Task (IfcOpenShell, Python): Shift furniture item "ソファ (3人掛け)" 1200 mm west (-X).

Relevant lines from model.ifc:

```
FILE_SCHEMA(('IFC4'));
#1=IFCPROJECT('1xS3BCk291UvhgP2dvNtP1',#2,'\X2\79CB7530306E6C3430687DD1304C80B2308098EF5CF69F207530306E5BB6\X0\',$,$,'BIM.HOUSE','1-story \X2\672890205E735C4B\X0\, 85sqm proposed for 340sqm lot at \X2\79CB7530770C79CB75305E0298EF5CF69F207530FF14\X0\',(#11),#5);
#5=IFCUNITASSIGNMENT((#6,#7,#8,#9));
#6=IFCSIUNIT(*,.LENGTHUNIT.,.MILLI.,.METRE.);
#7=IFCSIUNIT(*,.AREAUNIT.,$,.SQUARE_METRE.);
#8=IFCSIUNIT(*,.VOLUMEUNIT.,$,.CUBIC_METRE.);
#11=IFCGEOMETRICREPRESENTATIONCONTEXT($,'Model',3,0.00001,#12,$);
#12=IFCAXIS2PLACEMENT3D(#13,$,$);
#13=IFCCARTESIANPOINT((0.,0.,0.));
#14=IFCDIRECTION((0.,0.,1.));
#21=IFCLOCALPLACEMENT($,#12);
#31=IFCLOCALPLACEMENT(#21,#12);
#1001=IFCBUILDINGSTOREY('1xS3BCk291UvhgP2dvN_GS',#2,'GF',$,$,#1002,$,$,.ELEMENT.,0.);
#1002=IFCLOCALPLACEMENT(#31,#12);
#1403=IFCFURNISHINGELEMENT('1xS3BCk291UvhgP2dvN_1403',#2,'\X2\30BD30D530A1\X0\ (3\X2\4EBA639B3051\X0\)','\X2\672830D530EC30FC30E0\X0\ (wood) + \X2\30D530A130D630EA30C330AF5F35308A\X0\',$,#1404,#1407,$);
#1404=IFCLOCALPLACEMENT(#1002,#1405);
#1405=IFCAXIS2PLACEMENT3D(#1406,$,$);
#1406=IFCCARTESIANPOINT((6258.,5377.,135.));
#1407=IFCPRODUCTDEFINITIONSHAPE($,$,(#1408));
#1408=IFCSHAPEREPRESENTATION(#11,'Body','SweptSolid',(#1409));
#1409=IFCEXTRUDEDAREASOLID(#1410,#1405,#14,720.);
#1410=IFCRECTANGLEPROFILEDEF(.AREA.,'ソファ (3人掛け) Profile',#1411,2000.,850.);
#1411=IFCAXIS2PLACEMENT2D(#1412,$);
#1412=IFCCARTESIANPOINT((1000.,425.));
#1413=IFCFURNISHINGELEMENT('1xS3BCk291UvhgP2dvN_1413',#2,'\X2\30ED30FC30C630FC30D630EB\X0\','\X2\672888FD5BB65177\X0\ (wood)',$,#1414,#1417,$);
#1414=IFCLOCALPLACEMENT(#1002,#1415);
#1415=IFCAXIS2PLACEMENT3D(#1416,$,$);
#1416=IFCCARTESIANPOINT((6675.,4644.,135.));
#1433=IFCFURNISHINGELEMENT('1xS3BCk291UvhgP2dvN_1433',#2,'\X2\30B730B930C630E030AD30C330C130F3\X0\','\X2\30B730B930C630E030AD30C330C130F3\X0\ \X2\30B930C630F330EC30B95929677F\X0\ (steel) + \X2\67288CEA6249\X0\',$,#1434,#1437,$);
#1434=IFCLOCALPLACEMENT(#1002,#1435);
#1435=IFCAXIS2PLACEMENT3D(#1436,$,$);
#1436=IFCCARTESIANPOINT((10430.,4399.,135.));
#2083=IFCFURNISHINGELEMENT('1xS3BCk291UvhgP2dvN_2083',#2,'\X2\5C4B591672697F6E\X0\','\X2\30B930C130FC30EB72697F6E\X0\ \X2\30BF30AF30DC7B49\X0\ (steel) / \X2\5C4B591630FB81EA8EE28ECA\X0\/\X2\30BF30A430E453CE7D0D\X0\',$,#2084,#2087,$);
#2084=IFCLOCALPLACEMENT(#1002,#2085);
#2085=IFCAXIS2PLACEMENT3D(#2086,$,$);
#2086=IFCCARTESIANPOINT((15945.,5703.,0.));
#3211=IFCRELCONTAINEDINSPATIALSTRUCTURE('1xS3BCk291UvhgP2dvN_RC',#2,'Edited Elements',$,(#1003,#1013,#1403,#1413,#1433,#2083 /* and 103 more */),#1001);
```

```python
import ifcopenshell
import ifcopenshell.api.geometry
import ifcopenshell.util.placement
import ifcopenshell.util.unit

model = ifcopenshell.open("model.ifc")
unit_scale = ifcopenshell.util.unit.calculate_unit_scale(model)

item = model.by_guid("1xS3BCk291UvhgP2dvN_1403")
matrix = ifcopenshell.util.placement.get_local_placement(item.ObjectPlacement)
matrix[0, 3] -= 1.2 / unit_scale
ifcopenshell.api.geometry.edit_object_placement(model, product=item, matrix=matrix, is_si=False)

print(ifcopenshell.util.placement.get_local_placement(item.ObjectPlacement).round(3) + 0.0)

model.write("model_v2.ifc")
```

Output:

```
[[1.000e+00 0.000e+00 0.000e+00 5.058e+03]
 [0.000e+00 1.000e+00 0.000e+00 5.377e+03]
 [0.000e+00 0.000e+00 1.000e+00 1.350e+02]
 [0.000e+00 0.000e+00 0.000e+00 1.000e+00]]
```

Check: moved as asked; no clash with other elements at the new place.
